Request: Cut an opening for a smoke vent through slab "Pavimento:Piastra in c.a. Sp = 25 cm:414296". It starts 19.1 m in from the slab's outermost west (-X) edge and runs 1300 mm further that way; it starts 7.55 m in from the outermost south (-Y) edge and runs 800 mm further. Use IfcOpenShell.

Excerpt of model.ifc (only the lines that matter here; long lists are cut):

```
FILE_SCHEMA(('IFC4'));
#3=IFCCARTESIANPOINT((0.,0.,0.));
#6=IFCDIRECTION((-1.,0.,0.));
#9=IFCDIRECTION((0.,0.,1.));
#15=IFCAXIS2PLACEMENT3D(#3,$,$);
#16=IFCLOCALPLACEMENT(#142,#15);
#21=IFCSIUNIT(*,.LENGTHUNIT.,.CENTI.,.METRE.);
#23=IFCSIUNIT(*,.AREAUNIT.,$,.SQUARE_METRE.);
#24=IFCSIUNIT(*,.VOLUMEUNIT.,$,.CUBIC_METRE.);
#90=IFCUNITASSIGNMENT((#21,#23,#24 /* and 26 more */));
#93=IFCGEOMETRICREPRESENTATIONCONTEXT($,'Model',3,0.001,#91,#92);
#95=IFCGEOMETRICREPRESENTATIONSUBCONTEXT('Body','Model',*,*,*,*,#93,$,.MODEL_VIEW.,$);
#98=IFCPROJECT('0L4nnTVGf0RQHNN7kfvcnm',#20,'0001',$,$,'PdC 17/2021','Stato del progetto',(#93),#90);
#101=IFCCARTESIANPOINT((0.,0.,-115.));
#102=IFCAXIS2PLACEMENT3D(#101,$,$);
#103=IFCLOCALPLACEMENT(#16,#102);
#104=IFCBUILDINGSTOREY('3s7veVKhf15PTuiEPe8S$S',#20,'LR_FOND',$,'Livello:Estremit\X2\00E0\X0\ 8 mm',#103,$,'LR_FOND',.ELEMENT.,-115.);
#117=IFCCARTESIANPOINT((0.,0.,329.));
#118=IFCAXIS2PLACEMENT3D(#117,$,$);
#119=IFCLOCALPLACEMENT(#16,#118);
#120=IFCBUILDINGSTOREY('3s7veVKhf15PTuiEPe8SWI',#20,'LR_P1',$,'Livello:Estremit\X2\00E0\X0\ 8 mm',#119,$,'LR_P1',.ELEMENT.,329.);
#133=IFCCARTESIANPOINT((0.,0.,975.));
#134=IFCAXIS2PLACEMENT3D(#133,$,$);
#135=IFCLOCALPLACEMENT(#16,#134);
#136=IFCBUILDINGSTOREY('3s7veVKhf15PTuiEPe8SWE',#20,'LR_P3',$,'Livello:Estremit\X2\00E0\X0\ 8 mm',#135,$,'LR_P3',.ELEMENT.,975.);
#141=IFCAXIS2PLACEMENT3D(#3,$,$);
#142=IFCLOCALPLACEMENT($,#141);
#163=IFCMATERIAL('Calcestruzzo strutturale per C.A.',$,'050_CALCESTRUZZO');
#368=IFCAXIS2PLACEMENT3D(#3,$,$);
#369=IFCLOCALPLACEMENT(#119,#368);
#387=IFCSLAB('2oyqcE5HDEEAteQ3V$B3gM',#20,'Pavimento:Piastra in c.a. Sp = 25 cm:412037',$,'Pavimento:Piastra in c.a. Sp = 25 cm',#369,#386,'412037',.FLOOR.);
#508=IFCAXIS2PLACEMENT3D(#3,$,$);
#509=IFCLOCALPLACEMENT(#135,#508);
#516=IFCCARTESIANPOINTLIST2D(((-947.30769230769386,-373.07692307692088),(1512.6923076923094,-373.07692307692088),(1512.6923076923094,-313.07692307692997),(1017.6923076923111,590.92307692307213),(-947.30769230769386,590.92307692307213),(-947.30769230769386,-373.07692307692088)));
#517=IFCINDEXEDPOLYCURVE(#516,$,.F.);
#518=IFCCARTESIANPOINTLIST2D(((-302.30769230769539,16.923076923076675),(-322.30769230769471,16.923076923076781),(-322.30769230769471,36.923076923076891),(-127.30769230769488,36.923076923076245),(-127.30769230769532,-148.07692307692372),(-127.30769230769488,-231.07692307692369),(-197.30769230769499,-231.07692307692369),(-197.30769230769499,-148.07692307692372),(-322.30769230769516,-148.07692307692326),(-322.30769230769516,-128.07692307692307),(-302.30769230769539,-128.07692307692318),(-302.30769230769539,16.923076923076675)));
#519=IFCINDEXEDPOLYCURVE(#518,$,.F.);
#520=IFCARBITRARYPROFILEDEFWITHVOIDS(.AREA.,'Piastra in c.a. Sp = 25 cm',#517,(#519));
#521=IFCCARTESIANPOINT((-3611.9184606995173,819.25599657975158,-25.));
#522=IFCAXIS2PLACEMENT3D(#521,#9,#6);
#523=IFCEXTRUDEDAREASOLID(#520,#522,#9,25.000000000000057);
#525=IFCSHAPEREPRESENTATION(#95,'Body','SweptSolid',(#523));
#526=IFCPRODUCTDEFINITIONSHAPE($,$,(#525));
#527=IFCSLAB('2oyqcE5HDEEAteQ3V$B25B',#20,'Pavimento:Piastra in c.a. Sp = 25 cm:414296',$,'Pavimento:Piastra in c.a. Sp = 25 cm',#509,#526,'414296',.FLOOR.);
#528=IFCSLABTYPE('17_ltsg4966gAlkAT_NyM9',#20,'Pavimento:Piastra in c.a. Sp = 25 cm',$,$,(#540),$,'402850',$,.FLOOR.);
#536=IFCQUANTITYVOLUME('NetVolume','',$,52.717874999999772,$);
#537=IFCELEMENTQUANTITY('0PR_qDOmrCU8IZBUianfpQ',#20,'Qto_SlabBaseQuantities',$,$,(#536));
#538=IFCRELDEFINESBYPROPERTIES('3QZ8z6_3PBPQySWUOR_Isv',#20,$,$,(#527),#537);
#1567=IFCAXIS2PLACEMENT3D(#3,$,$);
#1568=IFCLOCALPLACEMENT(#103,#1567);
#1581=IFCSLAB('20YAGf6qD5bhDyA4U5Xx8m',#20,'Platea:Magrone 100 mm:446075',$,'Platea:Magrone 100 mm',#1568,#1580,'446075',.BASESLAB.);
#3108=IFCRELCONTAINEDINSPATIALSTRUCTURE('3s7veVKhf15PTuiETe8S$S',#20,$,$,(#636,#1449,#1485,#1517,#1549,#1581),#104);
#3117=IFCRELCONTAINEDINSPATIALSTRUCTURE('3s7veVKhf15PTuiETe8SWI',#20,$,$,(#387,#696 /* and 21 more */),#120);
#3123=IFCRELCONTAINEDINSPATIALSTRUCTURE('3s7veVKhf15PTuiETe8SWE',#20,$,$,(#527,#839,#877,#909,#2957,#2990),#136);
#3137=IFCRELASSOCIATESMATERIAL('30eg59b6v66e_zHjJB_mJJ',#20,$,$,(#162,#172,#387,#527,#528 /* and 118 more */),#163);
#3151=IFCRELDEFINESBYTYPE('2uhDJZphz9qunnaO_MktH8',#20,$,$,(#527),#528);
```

```python
import numpy as np
import ifcopenshell
import ifcopenshell.api.feature
import ifcopenshell.api.geometry
import ifcopenshell.api.pset
import ifcopenshell.api.root
import ifcopenshell.geom
import ifcopenshell.util.element
import ifcopenshell.util.placement
import ifcopenshell.util.representation
import ifcopenshell.util.shape
import ifcopenshell.util.unit

model = ifcopenshell.open("model.ifc")
unit_scale = ifcopenshell.util.unit.calculate_unit_scale(model)
volume_scale = ifcopenshell.util.unit.calculate_unit_scale(model, "VOLUMEUNIT")
settings = ifcopenshell.geom.settings()


def volume(element):
    """Net volume in cubic metres, openings subtracted."""
    shape = ifcopenshell.geom.create_shape(settings, element)
    return ifcopenshell.util.shape.get_volume(shape.geometry)


slab = model.by_guid("2oyqcE5HDEEAteQ3V$B25B")
before = volume(slab)

# Extent in the slab's own axes, in metres. The edges named are its -X and -Y sides.
slab_shape = ifcopenshell.geom.create_shape(settings, slab)
vertices = ifcopenshell.util.shape.get_vertices(slab_shape.geometry)
x_min, y_min, bottom = vertices.min(axis=0)
top = vertices[:, 2].max()

opening = ifcopenshell.api.root.create_entity(model, ifc_class="IfcOpeningElement", name="Smoke vent opening", predefined_type="OPENING")
context = ifcopenshell.util.representation.get_context(model, "Model", "Body", "MODEL_VIEW")
width, depth = 1.3, 0.8
outline = [(0.0, 0.0), (width, 0.0), (width, depth), (0.0, depth), (0.0, 0.0)]
# Overshoot both faces by 50 mm so the cut is clean.
shape = ifcopenshell.api.geometry.add_slab_representation(
    model, context=context, depth=top - bottom + 0.1, polyline=outline
)
ifcopenshell.api.geometry.assign_representation(model, product=opening, representation=shape)

matrix = ifcopenshell.util.placement.get_local_placement(slab.ObjectPlacement)
matrix[:, 3] = matrix @ np.append(np.array([x_min + 19.1, y_min + 7.55, bottom - 0.05]) / unit_scale, 1.0)
ifcopenshell.api.geometry.edit_object_placement(model, product=opening, matrix=matrix, is_si=False)
ifcopenshell.api.feature.add_feature(model, feature=opening, element=slab)

after = volume(slab)

# Update the slab's stored quantities.
qto = model.by_id(ifcopenshell.util.element.get_pset(slab, "Qto_SlabBaseQuantities", should_inherit=False)["id"])
ifcopenshell.api.pset.edit_qto(model, qto=qto, properties={"NetVolume": after / volume_scale})

print(f"slab volume {before:.3f} -> {after:.3f} m3")

model.write("model-out.ifc")
```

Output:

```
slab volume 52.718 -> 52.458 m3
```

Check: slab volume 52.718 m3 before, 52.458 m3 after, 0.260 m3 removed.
